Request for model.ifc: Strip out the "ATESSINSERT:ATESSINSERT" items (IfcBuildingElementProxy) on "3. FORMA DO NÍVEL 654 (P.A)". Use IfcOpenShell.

First a look at what the model holds.

```python
import ifcopenshell
import ifcopenshell.util.element

model = ifcopenshell.open("model.ifc")
print(model.schema)
storey = next(s for s in model.by_type("IfcBuildingStorey") if s.Name == "3. FORMA DO NÍVEL 654 (P.A)")
proxies = [e for e in ifcopenshell.util.element.get_decomposition(storey) if e.is_a("IfcBuildingElementProxy")]
seen = {}
for e in proxies:
    element_type = ifcopenshell.util.element.get_type(e)
    name = element_type.Name if element_type not in (None, e) else None
    seen[name] = seen.get(name, 0) + 1
for name, count in sorted(seen.items(), key=str):
    print(count, "x", name)
```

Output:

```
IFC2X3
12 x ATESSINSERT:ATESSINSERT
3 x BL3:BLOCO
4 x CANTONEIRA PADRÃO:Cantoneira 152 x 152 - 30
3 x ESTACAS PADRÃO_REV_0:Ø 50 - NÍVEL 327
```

```python
import ifcopenshell
import ifcopenshell.api.root
import ifcopenshell.util.element

model = ifcopenshell.open("model.ifc")

storey = next(s for s in model.by_type("IfcBuildingStorey") if s.Name == "3. FORMA DO NÍVEL 654 (P.A)")
proxies = [e for e in ifcopenshell.util.element.get_decomposition(storey) if e.is_a("IfcBuildingElementProxy")]
targets = [e for e in proxies if (t := ifcopenshell.util.element.get_type(e)) not in (None, e) and t.Name == "ATESSINSERT:ATESSINSERT"]

for e in targets:
    ifcopenshell.api.root.remove_product(model, product=e)
print(len(targets), "removed")

model.write("model_v2.ifc")
```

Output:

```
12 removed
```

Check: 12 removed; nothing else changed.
